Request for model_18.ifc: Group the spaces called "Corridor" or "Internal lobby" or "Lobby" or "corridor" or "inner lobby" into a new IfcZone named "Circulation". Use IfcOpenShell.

First a look at what the model holds.

```python
import ifcopenshell

model = ifcopenshell.open("model_18.ifc")
print(model.schema)
seen = {}
for space in model.by_type("IfcSpace"):
    seen[space.LongName] = seen.get(space.LongName, 0) + 1
for name, count in sorted(seen.items(), key=str):
    print(count, "x", name)
print("zones:", [z.Name for z in model.by_type("IfcZone")][:20])
```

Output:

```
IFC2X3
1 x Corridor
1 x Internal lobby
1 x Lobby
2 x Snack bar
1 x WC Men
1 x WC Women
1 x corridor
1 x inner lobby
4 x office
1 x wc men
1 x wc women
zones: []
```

```python
import ifcopenshell
import ifcopenshell.api.group
import ifcopenshell.api.root

model = ifcopenshell.open("model_18.ifc")

names = {"Corridor", "Internal lobby", "Lobby", "corridor", "inner lobby"}
spaces = [s for s in model.by_type("IfcSpace") if s.LongName in names]

zone = ifcopenshell.api.root.create_entity(model, ifc_class="IfcZone", name="Circulation")
ifcopenshell.api.group.assign_group(model, products=spaces, group=zone)
print(len(spaces), "spaces in", zone.Name)

model.write("model_18-out.ifc")
```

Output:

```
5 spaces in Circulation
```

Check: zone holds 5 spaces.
